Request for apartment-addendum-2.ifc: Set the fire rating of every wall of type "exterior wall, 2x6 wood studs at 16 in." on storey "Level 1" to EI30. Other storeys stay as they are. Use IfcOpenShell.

First a look at what the model holds.

```python
import ifcopenshell
import ifcopenshell.util.element

model = ifcopenshell.open("apartment-addendum-2.ifc")
print(model.schema)
storey = next(s for s in model.by_type("IfcBuildingStorey") if s.Name == "Level 1")
walls = [e for e in ifcopenshell.util.element.get_decomposition(storey) if e.is_a("IfcWall")]
seen = {}
for e in walls:
    element_type = ifcopenshell.util.element.get_type(e)
    key = (element_type.Name if element_type != e and element_type else None, ifcopenshell.util.element.get_pset(e, "Pset_WallCommon", "FireRating"))
    seen[key] = seen.get(key, 0) + 1
for (name, value), count in sorted(seen.items(), key=str):
    print(count, "x", name, "|", value)
```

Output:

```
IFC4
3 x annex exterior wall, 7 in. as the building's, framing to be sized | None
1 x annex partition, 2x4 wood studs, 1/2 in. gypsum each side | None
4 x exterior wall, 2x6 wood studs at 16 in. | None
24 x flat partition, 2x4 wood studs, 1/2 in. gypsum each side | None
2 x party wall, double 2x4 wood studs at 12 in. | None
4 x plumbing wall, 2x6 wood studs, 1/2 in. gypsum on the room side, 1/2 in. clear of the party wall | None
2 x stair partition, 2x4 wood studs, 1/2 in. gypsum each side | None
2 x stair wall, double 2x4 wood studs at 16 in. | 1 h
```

```python
import ifcopenshell
import ifcopenshell.api.pset
import ifcopenshell.util.element

model = ifcopenshell.open("apartment-addendum-2.ifc")

storey = next(s for s in model.by_type("IfcBuildingStorey") if s.Name == "Level 1")
walls = [e for e in ifcopenshell.util.element.get_decomposition(storey) if e.is_a("IfcWall")]

count = 0
for e in walls:
    element_type = ifcopenshell.util.element.get_type(e)
    if element_type in (None, e) or element_type.Name != "exterior wall, 2x6 wood studs at 16 in.":
        continue
    # add_pset returns the element's existing set when there is one.
    pset = ifcopenshell.api.pset.add_pset(model, product=e, name="Pset_WallCommon")
    ifcopenshell.api.pset.edit_pset(model, pset=pset, properties={"FireRating": "EI30"})
    count += 1

print(count, "walls updated")

model.write("apartment-addendum-2_rev.ifc")
```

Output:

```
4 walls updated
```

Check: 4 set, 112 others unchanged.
